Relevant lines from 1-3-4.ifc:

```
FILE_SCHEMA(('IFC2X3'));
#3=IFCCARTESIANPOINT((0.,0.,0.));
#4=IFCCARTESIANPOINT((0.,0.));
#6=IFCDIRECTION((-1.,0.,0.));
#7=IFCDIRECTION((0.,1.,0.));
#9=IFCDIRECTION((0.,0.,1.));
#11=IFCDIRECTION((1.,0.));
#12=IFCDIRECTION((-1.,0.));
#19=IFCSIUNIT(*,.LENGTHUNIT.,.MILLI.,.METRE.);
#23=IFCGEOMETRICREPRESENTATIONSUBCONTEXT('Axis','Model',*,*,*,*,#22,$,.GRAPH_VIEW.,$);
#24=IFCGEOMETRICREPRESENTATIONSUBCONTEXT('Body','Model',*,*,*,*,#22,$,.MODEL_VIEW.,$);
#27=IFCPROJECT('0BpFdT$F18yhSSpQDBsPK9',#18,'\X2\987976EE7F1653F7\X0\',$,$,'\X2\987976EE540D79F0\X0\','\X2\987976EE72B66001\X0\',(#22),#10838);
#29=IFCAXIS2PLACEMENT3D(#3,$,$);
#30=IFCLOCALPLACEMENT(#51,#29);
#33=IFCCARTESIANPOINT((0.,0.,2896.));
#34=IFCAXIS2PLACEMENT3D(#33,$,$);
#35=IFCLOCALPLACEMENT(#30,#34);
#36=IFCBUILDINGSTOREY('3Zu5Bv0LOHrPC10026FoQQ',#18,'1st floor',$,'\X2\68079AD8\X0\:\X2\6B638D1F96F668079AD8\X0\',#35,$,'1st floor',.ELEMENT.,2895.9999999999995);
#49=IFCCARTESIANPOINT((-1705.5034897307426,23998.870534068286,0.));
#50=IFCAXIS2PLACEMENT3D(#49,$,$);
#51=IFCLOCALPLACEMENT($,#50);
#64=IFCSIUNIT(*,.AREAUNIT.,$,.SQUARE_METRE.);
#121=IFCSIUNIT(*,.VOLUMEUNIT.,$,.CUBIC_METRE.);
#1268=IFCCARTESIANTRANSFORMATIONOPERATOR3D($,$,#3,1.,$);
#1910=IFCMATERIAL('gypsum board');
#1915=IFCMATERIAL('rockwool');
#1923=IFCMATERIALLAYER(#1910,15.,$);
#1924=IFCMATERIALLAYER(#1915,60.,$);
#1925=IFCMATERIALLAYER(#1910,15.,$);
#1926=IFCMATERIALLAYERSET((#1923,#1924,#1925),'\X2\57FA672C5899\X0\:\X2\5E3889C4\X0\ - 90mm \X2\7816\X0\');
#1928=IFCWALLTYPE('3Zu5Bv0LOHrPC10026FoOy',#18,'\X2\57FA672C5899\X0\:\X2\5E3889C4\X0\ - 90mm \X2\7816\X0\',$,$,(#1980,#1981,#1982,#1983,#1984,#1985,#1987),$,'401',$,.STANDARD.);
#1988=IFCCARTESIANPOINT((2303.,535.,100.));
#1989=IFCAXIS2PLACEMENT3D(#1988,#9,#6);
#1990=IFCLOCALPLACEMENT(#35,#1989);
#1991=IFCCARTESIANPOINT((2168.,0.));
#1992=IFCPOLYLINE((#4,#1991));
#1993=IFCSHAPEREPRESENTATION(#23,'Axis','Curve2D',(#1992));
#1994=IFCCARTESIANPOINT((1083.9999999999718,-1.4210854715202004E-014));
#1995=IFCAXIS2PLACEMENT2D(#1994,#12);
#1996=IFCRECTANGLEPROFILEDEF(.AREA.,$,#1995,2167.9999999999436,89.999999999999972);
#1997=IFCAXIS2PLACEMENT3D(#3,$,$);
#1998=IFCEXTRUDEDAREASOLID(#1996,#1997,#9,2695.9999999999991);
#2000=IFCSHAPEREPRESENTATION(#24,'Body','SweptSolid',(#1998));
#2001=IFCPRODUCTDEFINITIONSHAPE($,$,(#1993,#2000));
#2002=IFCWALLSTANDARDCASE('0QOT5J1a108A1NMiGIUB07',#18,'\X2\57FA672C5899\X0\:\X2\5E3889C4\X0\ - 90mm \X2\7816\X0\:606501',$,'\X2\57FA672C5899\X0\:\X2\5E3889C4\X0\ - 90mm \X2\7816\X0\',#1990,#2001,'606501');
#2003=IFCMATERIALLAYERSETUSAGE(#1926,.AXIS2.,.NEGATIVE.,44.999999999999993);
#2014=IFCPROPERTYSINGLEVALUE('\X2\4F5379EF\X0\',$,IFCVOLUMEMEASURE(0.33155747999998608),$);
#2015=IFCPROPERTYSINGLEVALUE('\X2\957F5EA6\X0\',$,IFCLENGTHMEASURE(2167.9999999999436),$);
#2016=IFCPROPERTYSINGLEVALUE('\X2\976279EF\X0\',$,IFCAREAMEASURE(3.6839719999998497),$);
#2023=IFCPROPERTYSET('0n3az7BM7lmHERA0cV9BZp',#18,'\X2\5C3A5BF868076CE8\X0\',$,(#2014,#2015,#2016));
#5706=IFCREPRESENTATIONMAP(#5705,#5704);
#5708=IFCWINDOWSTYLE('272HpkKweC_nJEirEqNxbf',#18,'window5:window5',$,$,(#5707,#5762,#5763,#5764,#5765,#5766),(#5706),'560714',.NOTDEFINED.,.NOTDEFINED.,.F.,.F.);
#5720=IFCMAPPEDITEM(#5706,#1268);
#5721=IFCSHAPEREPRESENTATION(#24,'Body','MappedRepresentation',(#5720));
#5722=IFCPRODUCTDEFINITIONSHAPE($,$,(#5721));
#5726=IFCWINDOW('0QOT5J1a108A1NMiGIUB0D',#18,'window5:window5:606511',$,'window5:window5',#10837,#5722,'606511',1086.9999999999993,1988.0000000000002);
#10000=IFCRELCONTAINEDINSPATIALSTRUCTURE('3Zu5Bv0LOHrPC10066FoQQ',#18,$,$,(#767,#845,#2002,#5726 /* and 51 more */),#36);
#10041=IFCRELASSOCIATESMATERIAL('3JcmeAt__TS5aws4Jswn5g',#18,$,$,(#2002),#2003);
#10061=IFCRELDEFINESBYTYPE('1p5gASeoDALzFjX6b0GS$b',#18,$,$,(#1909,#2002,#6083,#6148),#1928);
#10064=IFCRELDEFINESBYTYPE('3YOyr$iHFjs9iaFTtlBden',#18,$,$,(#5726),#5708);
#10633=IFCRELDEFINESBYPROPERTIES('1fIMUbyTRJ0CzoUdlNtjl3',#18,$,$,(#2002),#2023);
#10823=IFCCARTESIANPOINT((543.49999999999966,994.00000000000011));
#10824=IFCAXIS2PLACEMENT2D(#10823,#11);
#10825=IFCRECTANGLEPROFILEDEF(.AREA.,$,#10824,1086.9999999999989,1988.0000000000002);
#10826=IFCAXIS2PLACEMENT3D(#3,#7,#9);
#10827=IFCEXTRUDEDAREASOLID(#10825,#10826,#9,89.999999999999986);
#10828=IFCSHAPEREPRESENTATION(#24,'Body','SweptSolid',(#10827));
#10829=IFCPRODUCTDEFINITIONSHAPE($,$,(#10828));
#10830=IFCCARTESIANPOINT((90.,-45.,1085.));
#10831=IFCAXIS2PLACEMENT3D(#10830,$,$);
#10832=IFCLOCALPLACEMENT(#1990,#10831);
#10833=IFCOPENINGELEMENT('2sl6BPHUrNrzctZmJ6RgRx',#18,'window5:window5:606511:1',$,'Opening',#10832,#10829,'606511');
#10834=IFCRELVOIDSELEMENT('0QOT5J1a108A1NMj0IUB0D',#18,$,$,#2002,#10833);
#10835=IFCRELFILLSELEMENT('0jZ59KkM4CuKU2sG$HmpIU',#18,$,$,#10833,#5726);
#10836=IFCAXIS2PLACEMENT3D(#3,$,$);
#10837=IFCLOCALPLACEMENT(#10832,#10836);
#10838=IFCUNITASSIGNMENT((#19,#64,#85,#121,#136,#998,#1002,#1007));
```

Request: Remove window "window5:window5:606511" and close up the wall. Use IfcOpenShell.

```python
import ifcopenshell
import ifcopenshell.api.feature
import ifcopenshell.api.pset
import ifcopenshell.api.root
import ifcopenshell.geom
import ifcopenshell.util.element
import ifcopenshell.util.shape
import ifcopenshell.util.unit

model = ifcopenshell.open("1-3-4.ifc")
area_scale = ifcopenshell.util.unit.calculate_unit_scale(model, "AREAUNIT")
volume_scale = ifcopenshell.util.unit.calculate_unit_scale(model, "VOLUMEUNIT")
settings = ifcopenshell.geom.settings()


def volume(element):
    """Net volume in cubic metres, openings subtracted."""
    shape = ifcopenshell.geom.create_shape(settings, element)
    return ifcopenshell.util.shape.get_volume(shape.geometry)


window = model.by_guid("0QOT5J1a108A1NMiGIUB0D")
opening = window.FillsVoids[0].RelatingOpeningElement
wall = opening.VoidsElements[0].RelatingBuildingElement
before = volume(wall)

ifcopenshell.api.root.remove_product(model, product=window)
ifcopenshell.api.feature.remove_feature(model, feature=opening)

after = volume(wall)
thickness = 0.09  # wall thickness in metres

# Update the wall's stored quantities.
pset = model.by_id(ifcopenshell.util.element.get_pset(wall, "尺寸标注", should_inherit=False)["id"])
ifcopenshell.api.pset.edit_pset(model, pset=pset, properties={
    "体积": model.create_entity("IfcVolumeMeasure", after / volume_scale),
    "面积": model.create_entity("IfcAreaMeasure", after / thickness / area_scale),
})

print(f"wall volume {before:.3f} -> {after:.3f} m3")

model.write("1-3-4_edited.ifc")
```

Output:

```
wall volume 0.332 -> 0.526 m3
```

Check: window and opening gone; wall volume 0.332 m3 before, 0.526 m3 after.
